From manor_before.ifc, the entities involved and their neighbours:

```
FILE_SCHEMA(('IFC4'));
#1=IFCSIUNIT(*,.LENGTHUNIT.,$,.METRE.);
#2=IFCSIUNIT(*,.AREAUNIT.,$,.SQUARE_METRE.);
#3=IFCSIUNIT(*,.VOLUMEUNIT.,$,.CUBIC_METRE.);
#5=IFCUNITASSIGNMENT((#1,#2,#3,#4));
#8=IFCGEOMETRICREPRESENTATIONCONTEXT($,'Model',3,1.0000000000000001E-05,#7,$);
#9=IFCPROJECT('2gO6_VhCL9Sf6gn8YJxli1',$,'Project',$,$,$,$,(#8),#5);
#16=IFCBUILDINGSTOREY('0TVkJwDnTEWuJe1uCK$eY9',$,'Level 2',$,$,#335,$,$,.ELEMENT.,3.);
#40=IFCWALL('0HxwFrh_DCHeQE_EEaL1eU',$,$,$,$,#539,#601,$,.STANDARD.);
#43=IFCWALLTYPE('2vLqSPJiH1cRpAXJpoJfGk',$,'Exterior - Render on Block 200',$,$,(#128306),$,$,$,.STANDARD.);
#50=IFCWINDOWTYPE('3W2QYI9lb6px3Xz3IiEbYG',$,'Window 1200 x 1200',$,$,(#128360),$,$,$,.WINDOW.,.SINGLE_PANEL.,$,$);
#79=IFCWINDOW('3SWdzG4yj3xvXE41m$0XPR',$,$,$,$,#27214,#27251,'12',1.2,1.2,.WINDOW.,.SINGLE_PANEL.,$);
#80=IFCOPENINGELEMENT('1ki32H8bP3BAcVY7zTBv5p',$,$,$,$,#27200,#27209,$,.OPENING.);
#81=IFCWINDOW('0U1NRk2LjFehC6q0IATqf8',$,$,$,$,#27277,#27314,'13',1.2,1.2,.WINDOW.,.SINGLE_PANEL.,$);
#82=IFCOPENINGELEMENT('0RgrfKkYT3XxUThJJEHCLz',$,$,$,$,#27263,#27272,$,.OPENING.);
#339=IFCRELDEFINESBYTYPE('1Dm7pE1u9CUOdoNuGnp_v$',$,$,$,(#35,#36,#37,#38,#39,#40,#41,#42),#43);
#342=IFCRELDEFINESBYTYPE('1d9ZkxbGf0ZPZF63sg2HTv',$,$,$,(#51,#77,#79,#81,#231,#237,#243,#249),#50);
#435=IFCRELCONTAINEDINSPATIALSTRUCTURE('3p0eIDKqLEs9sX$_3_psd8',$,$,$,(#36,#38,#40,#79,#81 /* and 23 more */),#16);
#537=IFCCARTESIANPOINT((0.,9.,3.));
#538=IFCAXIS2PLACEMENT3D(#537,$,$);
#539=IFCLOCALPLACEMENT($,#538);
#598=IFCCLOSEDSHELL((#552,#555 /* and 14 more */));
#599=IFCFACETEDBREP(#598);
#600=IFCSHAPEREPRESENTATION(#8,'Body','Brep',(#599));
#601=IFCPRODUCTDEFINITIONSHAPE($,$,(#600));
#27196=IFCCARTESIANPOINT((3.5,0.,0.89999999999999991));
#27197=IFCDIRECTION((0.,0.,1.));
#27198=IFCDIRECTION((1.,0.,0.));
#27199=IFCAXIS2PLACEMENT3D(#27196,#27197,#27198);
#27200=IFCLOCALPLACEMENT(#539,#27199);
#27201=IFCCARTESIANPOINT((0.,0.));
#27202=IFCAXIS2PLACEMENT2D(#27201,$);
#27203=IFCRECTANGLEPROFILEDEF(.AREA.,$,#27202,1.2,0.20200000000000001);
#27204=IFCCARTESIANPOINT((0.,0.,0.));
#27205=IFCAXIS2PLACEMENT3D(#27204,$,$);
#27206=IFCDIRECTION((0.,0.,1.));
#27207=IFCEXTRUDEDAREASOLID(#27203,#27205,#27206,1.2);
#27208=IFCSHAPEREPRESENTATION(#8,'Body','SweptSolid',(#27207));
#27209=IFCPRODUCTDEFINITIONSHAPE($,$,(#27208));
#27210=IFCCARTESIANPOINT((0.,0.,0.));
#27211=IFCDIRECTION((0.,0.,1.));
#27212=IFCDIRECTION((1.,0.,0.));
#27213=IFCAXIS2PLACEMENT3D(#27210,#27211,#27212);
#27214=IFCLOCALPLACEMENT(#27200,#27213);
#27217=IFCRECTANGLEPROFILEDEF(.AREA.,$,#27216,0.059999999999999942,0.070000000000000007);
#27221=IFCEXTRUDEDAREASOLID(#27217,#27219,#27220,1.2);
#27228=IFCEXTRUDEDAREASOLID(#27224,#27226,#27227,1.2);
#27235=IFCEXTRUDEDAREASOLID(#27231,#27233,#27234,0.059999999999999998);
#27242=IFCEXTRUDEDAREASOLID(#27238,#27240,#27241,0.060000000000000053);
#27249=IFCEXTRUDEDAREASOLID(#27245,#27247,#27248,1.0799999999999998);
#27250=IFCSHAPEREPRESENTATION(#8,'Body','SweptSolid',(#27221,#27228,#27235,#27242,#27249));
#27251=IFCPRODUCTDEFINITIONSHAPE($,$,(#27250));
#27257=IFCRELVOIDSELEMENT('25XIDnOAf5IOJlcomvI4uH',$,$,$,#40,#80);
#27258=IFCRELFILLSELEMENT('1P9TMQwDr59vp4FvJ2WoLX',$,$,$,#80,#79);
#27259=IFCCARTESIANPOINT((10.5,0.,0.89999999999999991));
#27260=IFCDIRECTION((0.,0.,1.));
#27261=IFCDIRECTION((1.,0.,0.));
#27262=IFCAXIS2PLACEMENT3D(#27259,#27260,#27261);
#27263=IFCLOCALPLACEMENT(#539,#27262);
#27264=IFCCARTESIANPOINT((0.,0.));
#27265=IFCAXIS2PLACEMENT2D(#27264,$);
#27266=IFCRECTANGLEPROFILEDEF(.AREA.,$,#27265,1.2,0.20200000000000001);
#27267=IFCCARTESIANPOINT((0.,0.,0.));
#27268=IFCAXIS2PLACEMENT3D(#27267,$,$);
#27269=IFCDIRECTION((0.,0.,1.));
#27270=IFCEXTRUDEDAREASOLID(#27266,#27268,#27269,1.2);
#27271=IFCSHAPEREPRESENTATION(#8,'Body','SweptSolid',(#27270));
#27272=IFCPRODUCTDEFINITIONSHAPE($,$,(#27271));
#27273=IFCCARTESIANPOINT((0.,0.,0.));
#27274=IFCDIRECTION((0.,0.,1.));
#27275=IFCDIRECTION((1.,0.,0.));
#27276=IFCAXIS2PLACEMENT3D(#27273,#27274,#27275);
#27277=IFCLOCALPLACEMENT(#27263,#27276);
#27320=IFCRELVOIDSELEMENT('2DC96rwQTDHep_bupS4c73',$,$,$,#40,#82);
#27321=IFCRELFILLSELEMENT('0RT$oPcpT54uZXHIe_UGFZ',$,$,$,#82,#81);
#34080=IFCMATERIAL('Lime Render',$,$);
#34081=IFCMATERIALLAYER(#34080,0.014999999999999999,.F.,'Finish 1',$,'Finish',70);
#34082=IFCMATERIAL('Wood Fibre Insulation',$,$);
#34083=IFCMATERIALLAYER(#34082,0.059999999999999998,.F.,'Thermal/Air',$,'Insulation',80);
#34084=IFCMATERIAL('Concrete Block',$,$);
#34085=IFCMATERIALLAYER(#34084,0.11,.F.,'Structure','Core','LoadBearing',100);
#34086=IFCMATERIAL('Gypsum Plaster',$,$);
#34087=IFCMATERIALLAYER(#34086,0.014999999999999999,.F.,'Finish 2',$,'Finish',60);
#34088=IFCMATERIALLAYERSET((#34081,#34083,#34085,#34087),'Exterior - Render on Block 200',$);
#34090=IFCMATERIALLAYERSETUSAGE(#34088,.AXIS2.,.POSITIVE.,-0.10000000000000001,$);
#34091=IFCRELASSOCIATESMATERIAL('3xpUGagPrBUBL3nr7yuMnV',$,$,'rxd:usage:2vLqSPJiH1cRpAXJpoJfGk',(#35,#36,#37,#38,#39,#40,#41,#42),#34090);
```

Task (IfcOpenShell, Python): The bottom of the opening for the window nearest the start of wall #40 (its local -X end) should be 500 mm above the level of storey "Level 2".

```python
import numpy as np
import ifcopenshell
import ifcopenshell.api.geometry
import ifcopenshell.geom
import ifcopenshell.util.element
import ifcopenshell.util.placement
import ifcopenshell.util.shape
import ifcopenshell.util.unit

model = ifcopenshell.open("manor_before.ifc")
unit_scale = ifcopenshell.util.unit.calculate_unit_scale(model)

window = model.by_id(79)
opening = window.FillsVoids[0].RelatingOpeningElement
storey = ifcopenshell.util.element.get_container(window, ifc_class="IfcBuildingStorey")
level = ifcopenshell.util.placement.get_local_placement(storey.ObjectPlacement)[2, 3]

# The opening's origin need not be at the sill, so measure its lowest point.
shape = ifcopenshell.geom.create_shape(ifcopenshell.geom.settings(), opening)
bottom = ifcopenshell.util.shape.get_shape_bottom_elevation(shape, shape.geometry) / unit_scale
dz = level + 0.5 - bottom

shift = np.array([0.0, 0.0, dz])
# The window is placed relative to its opening, so it follows when the opening moves.
matrix = ifcopenshell.util.placement.get_local_placement(opening.ObjectPlacement)
matrix[:3, 3] += shift
ifcopenshell.api.geometry.edit_object_placement(
    model, product=opening, matrix=matrix, is_si=False, should_transform_children=True
)

print(f"moved by {dz * unit_scale:+.3f} m")

model.write("manor_before_updated.ifc")
```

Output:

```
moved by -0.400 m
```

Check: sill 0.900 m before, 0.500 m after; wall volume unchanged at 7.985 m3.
